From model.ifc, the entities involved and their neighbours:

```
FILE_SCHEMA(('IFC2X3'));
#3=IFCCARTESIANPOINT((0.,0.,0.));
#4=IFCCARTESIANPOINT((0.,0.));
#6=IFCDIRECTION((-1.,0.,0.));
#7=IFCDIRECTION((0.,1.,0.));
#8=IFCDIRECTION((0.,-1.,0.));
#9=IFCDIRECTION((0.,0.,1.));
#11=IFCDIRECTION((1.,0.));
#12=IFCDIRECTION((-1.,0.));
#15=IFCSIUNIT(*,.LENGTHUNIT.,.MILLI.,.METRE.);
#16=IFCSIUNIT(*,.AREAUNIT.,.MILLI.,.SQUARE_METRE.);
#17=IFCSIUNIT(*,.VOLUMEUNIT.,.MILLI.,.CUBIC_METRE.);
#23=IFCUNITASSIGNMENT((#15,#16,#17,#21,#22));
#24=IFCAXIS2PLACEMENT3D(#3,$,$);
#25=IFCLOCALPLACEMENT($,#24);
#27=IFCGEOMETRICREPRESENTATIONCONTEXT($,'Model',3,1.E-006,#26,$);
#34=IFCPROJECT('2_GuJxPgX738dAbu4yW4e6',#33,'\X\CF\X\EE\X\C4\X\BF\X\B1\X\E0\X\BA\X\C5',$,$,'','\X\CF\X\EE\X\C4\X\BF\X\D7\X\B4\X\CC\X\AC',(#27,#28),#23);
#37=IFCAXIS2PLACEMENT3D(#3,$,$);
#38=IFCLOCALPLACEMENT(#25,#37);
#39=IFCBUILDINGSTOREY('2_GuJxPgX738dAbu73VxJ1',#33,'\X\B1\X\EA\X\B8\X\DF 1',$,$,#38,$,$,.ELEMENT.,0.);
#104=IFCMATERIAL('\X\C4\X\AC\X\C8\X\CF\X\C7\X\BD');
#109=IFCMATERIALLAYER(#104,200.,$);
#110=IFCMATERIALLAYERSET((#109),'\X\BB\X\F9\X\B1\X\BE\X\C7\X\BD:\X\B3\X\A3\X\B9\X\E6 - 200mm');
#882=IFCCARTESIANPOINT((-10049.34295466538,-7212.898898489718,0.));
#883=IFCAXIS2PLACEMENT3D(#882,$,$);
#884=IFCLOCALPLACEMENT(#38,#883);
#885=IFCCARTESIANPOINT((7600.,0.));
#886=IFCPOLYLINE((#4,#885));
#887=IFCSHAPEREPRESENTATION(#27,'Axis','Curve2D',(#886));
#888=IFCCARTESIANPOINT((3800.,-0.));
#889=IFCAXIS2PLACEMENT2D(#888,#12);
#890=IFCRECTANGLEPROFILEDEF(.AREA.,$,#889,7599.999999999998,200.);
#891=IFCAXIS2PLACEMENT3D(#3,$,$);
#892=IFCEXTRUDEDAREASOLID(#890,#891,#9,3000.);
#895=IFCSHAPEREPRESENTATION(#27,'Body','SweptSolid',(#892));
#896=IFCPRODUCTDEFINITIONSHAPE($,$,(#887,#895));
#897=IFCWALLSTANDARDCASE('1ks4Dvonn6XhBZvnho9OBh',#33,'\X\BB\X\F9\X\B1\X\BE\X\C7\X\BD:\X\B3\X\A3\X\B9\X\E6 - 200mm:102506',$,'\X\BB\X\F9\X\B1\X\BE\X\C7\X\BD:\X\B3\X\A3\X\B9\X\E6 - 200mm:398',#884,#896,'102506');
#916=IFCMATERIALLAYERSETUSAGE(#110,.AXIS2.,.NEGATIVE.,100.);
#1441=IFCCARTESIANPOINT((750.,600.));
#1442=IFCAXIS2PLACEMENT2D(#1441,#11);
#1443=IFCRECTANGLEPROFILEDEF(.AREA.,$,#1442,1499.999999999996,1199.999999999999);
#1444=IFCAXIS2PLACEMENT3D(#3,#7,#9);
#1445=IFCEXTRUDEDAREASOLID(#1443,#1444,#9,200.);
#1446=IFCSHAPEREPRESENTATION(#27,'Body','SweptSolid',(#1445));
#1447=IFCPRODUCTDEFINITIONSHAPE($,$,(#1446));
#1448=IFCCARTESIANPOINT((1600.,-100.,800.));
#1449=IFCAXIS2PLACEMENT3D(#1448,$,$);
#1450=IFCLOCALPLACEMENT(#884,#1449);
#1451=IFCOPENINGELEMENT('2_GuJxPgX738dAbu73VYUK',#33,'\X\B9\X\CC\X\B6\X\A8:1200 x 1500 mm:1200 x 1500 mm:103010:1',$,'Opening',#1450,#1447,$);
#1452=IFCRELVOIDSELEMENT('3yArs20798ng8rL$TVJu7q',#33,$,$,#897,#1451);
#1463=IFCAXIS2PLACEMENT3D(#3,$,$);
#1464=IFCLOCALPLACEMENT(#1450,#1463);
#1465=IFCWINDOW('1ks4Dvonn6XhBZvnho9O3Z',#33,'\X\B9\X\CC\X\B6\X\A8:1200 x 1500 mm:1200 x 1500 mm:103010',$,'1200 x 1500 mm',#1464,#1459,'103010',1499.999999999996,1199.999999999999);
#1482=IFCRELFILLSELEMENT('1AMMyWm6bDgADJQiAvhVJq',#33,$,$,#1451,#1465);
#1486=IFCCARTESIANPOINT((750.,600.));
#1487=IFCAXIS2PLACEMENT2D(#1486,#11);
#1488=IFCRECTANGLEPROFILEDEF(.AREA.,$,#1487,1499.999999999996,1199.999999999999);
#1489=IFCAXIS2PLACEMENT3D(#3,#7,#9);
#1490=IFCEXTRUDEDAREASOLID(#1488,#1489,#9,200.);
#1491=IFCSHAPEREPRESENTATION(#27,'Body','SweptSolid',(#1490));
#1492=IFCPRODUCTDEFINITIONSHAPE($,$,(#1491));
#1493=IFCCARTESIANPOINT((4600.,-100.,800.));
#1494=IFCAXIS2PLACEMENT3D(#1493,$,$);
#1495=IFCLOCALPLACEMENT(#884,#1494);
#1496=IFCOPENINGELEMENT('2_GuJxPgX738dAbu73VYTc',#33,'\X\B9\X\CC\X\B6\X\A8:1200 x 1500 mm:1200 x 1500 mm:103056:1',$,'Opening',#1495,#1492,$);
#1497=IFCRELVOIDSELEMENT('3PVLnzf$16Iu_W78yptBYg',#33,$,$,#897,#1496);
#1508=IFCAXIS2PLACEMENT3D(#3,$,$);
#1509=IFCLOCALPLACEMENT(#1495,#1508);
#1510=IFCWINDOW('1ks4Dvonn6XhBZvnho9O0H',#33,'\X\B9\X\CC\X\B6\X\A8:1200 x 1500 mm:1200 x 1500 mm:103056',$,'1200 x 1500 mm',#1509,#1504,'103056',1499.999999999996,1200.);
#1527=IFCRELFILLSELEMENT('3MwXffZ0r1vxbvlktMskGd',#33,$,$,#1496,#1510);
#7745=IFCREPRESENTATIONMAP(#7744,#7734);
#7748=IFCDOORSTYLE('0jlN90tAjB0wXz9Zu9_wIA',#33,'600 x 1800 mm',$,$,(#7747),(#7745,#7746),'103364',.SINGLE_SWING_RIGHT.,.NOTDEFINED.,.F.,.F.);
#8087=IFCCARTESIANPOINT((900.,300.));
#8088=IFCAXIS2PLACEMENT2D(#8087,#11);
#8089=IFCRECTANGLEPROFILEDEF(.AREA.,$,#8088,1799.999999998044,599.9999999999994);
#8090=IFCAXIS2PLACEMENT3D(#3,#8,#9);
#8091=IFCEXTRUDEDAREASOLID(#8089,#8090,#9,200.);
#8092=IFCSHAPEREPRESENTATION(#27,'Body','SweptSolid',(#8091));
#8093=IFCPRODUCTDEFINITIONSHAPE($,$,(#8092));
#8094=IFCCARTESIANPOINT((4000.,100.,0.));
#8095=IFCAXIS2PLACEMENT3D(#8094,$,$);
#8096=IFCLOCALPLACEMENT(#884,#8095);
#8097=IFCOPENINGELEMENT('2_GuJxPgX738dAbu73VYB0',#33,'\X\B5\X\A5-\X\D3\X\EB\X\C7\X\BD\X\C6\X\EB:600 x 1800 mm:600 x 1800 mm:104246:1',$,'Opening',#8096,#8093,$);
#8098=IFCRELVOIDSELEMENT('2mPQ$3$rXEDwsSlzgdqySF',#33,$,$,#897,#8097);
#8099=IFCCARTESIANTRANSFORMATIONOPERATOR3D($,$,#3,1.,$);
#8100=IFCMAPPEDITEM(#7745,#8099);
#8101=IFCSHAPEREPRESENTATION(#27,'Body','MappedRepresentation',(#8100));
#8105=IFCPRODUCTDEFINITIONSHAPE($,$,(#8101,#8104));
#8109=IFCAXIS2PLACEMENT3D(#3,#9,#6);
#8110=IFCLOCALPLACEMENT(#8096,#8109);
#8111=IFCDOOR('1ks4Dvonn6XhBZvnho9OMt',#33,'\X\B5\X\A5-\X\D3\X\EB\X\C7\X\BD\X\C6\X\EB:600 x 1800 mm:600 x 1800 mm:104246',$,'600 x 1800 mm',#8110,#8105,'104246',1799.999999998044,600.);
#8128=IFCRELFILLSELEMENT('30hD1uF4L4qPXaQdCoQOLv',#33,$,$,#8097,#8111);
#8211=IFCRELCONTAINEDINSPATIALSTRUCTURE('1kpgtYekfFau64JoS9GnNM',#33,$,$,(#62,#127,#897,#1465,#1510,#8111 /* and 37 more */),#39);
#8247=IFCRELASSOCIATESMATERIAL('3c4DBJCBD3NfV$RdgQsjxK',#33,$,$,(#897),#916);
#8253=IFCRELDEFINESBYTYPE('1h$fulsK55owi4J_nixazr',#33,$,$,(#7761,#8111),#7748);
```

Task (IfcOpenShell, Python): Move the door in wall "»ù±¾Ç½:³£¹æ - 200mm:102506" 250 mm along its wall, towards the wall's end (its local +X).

```python
import ifcopenshell
import ifcopenshell.api.geometry
import ifcopenshell.util.placement
import ifcopenshell.util.unit

model = ifcopenshell.open("model.ifc")
unit_scale = ifcopenshell.util.unit.calculate_unit_scale(model)

door = model.by_guid("1ks4Dvonn6XhBZvnho9OMt")
opening = door.FillsVoids[0].RelatingOpeningElement
wall = opening.VoidsElements[0].RelatingBuildingElement

wall_matrix = ifcopenshell.util.placement.get_local_placement(wall.ObjectPlacement)
shift = wall_matrix[:3, 0] * 0.25 / unit_scale
before = ifcopenshell.util.placement.get_local_placement(door.ObjectPlacement)[:3, 3].copy()

# The door is placed relative to its opening, so it follows when the opening moves.
matrix = ifcopenshell.util.placement.get_local_placement(opening.ObjectPlacement)
matrix[:3, 3] += shift
ifcopenshell.api.geometry.edit_object_placement(
    model, product=opening, matrix=matrix, is_si=False, should_transform_children=True
)

after = ifcopenshell.util.placement.get_local_placement(door.ObjectPlacement)[:3, 3]
print("door moved by", (after - before).round(3) + 0.0)

model.write("model_rev.ifc")
```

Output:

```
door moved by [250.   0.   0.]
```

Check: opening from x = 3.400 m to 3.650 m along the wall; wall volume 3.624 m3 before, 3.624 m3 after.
